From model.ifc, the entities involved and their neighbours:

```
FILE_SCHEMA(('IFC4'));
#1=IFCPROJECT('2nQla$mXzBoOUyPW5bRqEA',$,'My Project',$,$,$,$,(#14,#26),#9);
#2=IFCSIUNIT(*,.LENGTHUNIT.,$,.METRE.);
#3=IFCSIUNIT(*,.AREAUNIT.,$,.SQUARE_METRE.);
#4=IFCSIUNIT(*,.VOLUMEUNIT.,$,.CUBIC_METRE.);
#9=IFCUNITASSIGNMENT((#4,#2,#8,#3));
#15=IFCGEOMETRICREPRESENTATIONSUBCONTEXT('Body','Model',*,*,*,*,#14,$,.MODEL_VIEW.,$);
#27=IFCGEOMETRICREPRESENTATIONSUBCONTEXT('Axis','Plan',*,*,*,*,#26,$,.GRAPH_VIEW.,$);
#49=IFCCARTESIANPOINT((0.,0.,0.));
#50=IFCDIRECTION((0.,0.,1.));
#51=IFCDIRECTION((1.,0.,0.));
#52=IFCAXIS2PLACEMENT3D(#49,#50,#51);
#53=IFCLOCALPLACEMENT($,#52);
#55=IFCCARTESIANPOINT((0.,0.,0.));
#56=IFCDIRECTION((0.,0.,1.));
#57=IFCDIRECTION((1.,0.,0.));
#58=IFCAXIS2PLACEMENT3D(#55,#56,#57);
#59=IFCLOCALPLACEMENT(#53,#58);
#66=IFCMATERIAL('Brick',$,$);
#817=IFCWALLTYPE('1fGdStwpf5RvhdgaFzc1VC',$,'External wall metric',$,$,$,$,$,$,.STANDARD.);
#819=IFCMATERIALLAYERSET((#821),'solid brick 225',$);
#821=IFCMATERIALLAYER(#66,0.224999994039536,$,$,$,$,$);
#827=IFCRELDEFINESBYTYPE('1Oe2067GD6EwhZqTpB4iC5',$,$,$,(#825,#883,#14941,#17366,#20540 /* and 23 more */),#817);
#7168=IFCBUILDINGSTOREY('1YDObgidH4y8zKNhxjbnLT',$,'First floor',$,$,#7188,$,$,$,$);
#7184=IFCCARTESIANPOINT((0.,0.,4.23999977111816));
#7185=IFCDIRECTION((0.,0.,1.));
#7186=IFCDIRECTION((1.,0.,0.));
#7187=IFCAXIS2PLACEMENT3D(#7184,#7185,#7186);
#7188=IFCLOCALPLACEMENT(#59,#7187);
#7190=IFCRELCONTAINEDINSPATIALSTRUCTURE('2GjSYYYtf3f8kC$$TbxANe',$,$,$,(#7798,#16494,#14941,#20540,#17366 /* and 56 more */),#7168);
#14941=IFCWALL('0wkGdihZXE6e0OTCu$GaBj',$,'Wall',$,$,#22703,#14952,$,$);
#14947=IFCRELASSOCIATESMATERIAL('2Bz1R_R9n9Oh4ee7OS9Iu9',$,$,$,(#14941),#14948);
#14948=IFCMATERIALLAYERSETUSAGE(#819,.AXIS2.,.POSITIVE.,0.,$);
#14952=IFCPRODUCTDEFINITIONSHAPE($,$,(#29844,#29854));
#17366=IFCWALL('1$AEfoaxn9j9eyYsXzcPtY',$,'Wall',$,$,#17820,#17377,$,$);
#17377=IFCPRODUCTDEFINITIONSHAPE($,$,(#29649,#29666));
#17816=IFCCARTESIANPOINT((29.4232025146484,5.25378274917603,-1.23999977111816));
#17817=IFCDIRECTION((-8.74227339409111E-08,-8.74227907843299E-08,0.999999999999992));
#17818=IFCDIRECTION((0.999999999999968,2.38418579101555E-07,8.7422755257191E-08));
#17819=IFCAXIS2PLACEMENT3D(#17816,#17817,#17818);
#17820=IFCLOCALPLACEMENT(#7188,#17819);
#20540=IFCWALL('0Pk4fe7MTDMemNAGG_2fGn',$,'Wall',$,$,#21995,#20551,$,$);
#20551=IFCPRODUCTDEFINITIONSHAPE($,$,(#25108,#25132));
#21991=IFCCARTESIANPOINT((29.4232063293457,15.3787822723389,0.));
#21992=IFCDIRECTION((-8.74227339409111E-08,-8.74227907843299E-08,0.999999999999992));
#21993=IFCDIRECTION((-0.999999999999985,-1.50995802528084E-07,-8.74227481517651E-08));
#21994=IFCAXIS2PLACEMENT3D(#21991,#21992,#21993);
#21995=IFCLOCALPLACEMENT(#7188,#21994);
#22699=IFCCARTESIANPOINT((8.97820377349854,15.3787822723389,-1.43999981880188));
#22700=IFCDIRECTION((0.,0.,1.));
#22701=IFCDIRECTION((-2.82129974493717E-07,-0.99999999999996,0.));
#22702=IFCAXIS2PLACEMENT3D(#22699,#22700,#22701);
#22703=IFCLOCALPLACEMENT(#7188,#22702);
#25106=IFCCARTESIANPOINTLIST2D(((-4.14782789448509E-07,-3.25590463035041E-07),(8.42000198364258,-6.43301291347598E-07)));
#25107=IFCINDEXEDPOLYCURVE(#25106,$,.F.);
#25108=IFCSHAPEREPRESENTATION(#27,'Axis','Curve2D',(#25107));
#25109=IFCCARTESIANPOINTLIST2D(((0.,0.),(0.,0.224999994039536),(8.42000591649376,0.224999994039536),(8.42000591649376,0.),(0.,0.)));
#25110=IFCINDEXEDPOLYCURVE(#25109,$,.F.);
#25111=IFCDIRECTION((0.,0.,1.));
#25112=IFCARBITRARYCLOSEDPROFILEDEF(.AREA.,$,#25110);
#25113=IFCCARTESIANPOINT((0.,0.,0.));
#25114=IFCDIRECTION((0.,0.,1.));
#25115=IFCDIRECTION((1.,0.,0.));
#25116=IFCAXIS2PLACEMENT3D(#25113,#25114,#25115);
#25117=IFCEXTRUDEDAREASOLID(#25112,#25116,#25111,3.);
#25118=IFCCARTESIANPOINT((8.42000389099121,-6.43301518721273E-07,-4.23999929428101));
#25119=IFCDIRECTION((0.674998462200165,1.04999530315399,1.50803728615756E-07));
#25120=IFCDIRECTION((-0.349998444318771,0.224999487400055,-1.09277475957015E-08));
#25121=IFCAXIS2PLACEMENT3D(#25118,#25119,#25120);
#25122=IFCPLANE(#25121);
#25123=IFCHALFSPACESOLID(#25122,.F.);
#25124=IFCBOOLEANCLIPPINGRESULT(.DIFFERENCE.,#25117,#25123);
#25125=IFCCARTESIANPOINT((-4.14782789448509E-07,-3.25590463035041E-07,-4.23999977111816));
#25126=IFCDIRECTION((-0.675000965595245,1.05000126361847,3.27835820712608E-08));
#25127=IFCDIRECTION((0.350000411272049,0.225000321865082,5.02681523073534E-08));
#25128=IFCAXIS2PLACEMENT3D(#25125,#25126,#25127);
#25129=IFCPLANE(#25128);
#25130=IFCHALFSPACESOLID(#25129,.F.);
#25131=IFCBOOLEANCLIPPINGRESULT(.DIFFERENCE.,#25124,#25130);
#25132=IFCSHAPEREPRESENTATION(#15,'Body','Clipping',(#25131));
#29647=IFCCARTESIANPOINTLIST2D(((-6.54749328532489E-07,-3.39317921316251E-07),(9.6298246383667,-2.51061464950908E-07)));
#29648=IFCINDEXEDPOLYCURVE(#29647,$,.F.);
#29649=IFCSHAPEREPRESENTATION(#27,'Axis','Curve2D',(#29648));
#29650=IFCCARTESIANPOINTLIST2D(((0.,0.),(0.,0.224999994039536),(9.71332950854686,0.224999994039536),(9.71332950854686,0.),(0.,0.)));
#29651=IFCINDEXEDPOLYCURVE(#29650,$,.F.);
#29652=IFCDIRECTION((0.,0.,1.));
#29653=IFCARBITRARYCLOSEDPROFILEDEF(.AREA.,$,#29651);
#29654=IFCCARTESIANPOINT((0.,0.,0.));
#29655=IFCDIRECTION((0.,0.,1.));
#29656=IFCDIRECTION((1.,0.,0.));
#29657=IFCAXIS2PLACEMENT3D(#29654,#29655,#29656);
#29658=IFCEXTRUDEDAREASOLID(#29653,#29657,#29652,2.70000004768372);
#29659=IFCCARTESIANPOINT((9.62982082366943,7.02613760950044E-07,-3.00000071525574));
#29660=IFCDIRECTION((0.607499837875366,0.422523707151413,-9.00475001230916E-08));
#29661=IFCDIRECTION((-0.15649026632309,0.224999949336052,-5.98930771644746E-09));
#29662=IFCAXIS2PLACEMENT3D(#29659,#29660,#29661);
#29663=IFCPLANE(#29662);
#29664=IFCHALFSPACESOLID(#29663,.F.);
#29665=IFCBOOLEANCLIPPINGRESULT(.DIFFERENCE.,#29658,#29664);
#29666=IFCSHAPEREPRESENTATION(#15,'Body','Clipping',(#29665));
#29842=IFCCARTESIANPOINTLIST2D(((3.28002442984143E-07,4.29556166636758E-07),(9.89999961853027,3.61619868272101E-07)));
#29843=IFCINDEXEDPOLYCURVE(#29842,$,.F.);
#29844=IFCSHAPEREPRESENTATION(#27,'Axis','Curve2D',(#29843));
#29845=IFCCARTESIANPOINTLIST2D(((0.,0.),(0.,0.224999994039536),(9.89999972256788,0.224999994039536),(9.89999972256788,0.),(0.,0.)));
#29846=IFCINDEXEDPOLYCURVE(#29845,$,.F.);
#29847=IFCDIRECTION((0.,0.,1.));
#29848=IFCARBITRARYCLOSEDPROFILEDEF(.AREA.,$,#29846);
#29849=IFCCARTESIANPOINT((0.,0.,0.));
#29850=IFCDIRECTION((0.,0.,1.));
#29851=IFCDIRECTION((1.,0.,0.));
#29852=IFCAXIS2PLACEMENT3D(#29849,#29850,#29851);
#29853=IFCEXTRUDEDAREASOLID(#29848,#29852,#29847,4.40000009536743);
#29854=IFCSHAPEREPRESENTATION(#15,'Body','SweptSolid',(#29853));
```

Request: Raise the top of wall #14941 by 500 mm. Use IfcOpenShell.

```python
import ifcopenshell
import ifcopenshell.geom
import ifcopenshell.util.representation
import ifcopenshell.util.shape

model = ifcopenshell.open("model.ifc")
settings = ifcopenshell.geom.settings()


def volume(element):
    """Net volume in cubic metres, openings subtracted."""
    shape = ifcopenshell.geom.create_shape(settings, element)
    return ifcopenshell.util.shape.get_volume(shape.geometry)


wall = model.by_guid("0wkGdihZXE6e0OTCu$GaBj")
before = volume(wall)

body = ifcopenshell.util.representation.get_representation(wall, "Model", "Body")
solid = body.Items[0]
old_height = solid.Depth
solid.Depth += 0.5
after = volume(wall)

print(f"height {old_height:g} -> {solid.Depth:g}, volume {before:.3f} -> {after:.3f} m3")

model.write("model_updated.ifc")
```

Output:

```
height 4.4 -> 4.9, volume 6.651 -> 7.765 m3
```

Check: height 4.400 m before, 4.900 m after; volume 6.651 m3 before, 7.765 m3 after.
